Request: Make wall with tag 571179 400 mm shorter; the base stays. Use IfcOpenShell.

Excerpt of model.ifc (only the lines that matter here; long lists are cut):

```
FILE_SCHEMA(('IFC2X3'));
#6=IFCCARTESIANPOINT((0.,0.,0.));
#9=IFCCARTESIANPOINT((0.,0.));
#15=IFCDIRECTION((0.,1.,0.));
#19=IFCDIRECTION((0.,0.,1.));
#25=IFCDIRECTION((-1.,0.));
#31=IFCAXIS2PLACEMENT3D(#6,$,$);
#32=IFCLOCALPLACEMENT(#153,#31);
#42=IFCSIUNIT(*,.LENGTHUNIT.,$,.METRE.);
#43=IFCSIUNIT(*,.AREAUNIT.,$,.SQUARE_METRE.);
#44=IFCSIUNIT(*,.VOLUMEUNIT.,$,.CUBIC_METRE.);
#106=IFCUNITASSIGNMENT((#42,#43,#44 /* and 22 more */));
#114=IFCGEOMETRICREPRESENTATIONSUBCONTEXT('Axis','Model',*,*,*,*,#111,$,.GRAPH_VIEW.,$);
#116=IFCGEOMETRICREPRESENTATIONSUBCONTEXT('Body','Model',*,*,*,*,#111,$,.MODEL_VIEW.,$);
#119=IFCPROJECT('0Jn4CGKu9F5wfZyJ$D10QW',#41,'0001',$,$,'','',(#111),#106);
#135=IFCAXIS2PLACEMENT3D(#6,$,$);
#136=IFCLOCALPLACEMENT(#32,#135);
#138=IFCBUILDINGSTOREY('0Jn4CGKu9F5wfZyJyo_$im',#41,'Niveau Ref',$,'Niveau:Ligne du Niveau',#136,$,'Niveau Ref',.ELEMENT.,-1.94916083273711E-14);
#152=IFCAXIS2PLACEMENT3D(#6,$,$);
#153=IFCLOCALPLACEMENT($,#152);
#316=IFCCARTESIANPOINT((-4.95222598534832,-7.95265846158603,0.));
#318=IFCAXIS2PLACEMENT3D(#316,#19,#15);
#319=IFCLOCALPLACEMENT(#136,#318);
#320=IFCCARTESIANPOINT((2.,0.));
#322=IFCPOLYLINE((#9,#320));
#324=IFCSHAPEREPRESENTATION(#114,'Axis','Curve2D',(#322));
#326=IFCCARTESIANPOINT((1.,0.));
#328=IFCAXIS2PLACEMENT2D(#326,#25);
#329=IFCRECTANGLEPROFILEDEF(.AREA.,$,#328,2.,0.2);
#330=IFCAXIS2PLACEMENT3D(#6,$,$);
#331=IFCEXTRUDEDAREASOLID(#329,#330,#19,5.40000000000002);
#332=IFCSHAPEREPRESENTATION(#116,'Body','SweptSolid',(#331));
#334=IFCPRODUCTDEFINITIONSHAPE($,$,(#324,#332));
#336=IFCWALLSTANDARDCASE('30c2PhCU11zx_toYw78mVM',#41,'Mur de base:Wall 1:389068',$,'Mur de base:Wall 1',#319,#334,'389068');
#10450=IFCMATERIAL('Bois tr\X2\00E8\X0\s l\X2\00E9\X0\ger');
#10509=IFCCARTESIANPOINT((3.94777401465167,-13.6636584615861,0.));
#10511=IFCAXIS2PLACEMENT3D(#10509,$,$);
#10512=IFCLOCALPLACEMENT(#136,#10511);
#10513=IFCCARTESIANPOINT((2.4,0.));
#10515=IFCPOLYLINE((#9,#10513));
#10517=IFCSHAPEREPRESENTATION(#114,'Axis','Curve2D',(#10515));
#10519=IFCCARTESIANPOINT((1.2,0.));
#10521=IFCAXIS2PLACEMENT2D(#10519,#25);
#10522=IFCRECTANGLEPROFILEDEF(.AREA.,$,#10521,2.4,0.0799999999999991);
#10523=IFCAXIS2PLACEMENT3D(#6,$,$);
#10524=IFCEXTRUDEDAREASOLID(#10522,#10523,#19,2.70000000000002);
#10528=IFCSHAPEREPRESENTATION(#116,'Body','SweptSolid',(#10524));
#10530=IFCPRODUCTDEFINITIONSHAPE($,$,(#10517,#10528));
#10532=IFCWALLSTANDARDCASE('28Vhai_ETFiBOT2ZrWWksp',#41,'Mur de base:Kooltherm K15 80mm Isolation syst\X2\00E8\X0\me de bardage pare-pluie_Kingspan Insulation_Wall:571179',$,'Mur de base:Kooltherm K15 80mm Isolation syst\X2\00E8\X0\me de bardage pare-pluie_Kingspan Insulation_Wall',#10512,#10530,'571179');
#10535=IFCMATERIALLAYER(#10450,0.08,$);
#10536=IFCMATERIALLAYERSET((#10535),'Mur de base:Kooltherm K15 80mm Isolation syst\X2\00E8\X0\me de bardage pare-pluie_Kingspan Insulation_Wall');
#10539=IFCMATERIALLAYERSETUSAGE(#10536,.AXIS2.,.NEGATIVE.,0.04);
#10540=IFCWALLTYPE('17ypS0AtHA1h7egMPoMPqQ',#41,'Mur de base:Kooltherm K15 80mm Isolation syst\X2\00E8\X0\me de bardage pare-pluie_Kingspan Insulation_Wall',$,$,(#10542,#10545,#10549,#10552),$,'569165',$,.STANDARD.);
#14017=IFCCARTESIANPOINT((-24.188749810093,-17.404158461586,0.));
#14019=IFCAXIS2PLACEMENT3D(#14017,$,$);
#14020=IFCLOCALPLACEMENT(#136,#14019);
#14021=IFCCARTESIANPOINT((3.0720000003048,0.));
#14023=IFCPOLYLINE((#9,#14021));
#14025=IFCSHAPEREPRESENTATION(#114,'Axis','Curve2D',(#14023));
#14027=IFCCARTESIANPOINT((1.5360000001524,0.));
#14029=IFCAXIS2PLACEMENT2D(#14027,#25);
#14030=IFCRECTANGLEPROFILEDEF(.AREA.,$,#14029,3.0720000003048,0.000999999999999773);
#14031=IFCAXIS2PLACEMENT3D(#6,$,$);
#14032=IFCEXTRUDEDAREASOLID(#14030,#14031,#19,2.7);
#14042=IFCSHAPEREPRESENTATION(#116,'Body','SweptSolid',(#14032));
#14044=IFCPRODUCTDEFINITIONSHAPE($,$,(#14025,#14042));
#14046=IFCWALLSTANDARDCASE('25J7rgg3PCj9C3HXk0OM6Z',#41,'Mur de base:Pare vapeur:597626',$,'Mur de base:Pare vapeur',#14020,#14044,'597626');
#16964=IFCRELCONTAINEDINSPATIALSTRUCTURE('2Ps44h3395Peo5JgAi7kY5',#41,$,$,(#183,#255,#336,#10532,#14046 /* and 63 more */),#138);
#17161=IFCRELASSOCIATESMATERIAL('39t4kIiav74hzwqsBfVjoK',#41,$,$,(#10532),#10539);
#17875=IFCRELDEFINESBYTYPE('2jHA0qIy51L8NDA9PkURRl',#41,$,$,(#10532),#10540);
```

```python
import ifcopenshell
import ifcopenshell.geom
import ifcopenshell.util.representation
import ifcopenshell.util.shape
import ifcopenshell.util.unit

model = ifcopenshell.open("model.ifc")
unit_scale = ifcopenshell.util.unit.calculate_unit_scale(model)
settings = ifcopenshell.geom.settings()


def volume(element):
    """Net volume in cubic metres, openings subtracted."""
    shape = ifcopenshell.geom.create_shape(settings, element)
    return ifcopenshell.util.shape.get_volume(shape.geometry)


wall = model.by_guid("28Vhai_ETFiBOT2ZrWWksp")
before = volume(wall)

body = ifcopenshell.util.representation.get_representation(wall, "Model", "Body")
solid = body.Items[0]
old_height = solid.Depth
solid.Depth -= 0.4 / unit_scale
after = volume(wall)

print(f"height {old_height:g} -> {solid.Depth:g}, volume {before:.3f} -> {after:.3f} m3")

model.write("model_v2.ifc")
```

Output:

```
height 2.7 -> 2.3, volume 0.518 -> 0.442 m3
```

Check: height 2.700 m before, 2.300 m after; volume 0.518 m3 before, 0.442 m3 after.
